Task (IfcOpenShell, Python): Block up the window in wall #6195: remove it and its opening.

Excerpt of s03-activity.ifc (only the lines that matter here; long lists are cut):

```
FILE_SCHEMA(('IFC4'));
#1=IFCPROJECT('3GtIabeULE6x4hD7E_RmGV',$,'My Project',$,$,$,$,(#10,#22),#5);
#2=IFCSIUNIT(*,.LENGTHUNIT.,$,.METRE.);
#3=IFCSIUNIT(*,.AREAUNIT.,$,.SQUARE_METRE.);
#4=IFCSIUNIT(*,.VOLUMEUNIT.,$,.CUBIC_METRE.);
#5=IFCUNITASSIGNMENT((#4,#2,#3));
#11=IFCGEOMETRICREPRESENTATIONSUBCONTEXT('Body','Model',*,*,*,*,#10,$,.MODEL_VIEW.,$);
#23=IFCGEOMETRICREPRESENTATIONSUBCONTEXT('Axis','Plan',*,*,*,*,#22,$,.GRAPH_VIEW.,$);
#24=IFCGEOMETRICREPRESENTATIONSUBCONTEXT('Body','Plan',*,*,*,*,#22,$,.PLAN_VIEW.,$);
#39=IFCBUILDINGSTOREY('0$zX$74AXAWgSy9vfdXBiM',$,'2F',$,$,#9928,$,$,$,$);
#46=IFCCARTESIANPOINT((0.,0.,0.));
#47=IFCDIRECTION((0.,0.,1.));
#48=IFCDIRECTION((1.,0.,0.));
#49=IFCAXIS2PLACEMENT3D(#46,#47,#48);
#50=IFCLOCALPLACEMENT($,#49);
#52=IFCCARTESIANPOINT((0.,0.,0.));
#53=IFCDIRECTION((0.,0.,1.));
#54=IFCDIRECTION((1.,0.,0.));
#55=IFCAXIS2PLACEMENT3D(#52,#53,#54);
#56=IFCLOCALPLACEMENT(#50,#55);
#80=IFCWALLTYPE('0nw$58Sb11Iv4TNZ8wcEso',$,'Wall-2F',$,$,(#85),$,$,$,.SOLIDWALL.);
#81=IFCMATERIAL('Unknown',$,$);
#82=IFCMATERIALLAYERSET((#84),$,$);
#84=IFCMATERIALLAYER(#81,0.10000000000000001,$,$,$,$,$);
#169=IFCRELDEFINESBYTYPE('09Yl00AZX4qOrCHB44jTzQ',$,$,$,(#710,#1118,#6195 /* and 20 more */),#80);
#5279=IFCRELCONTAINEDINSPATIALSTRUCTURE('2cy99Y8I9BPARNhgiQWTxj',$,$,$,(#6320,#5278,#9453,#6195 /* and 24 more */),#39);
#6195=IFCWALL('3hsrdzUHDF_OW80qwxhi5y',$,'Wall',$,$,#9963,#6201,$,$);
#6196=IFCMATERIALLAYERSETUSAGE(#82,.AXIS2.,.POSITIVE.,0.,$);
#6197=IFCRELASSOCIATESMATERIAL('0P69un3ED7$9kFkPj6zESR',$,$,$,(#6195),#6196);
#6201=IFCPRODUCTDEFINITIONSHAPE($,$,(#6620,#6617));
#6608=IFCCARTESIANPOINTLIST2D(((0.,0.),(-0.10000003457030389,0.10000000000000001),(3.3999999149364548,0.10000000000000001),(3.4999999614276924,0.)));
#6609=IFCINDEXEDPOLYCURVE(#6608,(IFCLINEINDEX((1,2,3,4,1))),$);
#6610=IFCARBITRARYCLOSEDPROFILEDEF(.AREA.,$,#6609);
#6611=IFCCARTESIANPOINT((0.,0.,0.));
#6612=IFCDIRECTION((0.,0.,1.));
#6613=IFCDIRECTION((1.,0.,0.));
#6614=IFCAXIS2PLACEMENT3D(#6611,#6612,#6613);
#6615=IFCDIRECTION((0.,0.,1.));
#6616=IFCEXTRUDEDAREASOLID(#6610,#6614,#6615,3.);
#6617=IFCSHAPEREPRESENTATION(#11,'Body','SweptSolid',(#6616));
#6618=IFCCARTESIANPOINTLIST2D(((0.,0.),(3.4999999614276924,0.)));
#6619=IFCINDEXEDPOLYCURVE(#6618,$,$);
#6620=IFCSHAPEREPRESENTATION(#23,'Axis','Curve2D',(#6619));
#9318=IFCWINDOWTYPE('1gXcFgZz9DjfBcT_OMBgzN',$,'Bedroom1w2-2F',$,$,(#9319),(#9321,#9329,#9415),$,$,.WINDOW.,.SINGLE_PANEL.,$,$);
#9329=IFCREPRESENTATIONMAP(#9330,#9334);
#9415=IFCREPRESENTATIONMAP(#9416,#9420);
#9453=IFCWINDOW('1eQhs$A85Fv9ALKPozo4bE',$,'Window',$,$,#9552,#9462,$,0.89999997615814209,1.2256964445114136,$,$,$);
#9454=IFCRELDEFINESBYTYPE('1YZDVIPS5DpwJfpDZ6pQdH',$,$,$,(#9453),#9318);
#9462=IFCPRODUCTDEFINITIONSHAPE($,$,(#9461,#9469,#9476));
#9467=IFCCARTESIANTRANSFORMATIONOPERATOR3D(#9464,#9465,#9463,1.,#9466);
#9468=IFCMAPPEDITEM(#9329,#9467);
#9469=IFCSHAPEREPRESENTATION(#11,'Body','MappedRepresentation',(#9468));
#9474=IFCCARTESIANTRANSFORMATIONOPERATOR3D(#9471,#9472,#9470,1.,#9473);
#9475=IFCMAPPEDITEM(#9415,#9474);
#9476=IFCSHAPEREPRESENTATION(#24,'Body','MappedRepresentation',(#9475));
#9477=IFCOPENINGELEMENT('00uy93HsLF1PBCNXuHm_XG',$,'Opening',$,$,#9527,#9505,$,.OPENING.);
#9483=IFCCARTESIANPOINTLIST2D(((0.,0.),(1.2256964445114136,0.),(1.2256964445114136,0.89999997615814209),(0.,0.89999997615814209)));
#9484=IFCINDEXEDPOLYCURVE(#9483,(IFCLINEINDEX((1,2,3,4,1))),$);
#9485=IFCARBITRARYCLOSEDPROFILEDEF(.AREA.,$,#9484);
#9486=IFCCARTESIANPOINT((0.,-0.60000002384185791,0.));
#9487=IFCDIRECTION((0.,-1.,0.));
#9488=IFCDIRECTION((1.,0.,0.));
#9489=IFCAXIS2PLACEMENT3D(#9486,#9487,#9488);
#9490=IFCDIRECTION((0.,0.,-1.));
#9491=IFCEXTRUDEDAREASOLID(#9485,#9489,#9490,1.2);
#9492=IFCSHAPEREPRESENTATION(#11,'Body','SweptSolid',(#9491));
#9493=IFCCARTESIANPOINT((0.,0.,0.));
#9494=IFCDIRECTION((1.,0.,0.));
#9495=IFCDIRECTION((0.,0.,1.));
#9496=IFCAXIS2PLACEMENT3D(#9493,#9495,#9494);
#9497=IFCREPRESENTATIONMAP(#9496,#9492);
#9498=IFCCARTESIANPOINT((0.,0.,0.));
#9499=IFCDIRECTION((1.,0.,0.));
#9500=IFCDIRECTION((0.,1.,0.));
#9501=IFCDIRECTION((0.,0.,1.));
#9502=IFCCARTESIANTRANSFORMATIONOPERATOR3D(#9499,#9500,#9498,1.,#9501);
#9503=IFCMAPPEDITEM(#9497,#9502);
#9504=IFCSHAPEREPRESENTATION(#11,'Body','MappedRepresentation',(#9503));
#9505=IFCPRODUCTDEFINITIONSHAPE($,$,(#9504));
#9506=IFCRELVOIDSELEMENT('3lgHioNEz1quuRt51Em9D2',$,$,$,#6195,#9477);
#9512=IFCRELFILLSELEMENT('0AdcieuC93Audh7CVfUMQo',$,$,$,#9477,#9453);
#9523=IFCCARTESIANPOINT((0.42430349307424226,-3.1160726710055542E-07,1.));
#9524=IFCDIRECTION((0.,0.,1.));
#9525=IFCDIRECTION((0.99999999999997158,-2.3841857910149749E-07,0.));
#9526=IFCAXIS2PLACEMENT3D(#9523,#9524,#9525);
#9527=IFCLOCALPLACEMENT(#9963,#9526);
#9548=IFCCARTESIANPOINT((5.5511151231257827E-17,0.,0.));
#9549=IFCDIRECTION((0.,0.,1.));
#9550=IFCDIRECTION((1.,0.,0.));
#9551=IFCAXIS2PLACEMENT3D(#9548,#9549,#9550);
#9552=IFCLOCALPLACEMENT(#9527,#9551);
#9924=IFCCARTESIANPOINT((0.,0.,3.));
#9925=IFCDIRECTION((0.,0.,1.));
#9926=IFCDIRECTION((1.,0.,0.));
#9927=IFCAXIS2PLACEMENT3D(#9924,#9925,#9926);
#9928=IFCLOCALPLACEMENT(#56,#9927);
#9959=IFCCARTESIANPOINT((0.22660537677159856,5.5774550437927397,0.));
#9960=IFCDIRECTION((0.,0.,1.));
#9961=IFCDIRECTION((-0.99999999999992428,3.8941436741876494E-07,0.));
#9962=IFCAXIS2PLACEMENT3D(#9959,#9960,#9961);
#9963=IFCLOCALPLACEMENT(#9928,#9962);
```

```python
import ifcopenshell
import ifcopenshell.api.feature
import ifcopenshell.api.root
import ifcopenshell.geom
import ifcopenshell.util.shape

model = ifcopenshell.open("s03-activity.ifc")
settings = ifcopenshell.geom.settings()


def volume(element):
    """Net volume in cubic metres, openings subtracted."""
    shape = ifcopenshell.geom.create_shape(settings, element)
    return ifcopenshell.util.shape.get_volume(shape.geometry)


window = model.by_id(9453)
opening = window.FillsVoids[0].RelatingOpeningElement
wall = opening.VoidsElements[0].RelatingBuildingElement
before = volume(wall)

ifcopenshell.api.root.remove_product(model, product=window)
ifcopenshell.api.feature.remove_feature(model, feature=opening)

after = volume(wall)

print(f"wall volume {before:.3f} -> {after:.3f} m3")

model.write("s03-activity_edited.ifc")
```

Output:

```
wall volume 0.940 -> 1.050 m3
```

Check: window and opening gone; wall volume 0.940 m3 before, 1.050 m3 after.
